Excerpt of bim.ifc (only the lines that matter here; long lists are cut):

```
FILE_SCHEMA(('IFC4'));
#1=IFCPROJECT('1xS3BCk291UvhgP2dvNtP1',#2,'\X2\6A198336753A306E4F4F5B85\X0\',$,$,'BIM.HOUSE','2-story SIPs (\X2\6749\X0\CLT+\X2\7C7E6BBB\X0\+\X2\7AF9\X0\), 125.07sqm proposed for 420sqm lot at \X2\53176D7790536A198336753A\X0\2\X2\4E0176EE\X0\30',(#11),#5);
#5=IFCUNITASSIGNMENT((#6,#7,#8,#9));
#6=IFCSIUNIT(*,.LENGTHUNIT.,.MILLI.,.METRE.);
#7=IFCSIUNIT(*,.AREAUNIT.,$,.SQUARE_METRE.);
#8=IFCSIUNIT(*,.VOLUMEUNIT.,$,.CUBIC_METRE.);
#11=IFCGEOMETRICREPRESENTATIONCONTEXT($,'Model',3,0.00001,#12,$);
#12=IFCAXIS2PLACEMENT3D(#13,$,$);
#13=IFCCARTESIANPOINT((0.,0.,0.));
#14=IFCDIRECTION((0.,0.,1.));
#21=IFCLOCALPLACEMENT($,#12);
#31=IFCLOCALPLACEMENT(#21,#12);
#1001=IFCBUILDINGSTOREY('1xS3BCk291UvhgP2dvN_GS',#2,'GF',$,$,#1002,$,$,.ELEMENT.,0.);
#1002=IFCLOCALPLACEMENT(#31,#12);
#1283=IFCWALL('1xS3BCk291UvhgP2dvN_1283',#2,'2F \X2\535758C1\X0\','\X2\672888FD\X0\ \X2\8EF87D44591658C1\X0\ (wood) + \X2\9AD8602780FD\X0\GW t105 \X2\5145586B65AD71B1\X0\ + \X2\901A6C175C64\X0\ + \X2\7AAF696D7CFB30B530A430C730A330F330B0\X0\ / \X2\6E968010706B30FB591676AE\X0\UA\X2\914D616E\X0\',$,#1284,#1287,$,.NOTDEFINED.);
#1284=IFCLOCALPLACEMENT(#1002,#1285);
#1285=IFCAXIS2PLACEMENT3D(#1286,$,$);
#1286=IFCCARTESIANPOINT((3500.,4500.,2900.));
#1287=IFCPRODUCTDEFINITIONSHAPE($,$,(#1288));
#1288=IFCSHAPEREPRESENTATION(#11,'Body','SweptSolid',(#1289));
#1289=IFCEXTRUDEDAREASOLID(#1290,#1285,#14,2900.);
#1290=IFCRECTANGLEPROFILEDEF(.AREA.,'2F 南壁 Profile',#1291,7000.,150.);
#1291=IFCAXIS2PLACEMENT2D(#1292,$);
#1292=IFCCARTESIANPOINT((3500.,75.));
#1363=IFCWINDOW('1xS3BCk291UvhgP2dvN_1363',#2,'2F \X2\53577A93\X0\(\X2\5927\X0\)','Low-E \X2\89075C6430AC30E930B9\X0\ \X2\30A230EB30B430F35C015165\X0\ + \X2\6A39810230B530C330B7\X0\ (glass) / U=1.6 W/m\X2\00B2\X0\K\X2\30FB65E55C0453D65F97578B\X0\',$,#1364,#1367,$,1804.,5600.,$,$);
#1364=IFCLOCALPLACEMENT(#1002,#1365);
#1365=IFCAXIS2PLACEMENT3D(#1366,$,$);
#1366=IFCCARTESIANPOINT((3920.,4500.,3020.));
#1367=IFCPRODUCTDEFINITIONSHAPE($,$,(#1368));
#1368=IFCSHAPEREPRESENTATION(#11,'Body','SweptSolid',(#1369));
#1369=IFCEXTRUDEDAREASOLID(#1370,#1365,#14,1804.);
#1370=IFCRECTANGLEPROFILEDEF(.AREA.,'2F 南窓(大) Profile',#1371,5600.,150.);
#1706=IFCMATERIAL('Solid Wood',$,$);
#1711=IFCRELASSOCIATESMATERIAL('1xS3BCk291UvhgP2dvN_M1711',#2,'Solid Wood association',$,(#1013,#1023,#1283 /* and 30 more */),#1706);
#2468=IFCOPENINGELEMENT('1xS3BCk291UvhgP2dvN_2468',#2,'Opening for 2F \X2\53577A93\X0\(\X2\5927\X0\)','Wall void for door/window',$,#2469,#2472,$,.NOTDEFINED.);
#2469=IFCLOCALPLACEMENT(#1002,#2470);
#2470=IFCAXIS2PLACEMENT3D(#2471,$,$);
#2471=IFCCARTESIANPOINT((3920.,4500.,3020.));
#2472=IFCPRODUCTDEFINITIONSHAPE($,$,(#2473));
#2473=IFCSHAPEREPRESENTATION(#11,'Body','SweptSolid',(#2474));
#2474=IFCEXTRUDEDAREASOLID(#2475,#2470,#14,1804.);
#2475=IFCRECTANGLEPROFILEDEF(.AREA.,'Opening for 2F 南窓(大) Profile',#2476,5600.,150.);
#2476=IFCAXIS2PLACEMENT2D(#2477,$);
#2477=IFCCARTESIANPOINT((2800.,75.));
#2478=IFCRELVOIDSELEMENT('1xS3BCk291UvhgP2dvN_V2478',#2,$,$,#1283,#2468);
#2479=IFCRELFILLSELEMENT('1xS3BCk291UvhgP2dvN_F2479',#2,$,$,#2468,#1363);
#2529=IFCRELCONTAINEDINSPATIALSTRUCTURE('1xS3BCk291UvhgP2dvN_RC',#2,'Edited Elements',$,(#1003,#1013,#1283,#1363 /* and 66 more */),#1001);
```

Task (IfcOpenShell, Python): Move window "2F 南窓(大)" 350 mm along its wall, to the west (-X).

```python
import ifcopenshell
import ifcopenshell.api.geometry
import ifcopenshell.util.placement

model = ifcopenshell.open("bim.ifc")

window = model.by_id(1363)
opening = window.FillsVoids[0].RelatingOpeningElement
wall = opening.VoidsElements[0].RelatingBuildingElement

wall_matrix = ifcopenshell.util.placement.get_local_placement(wall.ObjectPlacement)
shift = wall_matrix[:3, 0] * -350.0
before = ifcopenshell.util.placement.get_local_placement(window.ObjectPlacement)[:3, 3].copy()

# The window is not placed relative to its opening, so move both.
for product in (opening, window):
    matrix = ifcopenshell.util.placement.get_local_placement(product.ObjectPlacement)
    matrix[:3, 3] += shift
    ifcopenshell.api.geometry.edit_object_placement(model, product=product, matrix=matrix, is_si=False)

after = ifcopenshell.util.placement.get_local_placement(window.ObjectPlacement)[:3, 3]
print("window moved by", (after - before).round(3) + 0.0)

model.write("bim_edited.ifc")
```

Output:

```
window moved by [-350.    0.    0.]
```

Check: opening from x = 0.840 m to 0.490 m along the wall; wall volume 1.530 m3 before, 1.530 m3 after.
